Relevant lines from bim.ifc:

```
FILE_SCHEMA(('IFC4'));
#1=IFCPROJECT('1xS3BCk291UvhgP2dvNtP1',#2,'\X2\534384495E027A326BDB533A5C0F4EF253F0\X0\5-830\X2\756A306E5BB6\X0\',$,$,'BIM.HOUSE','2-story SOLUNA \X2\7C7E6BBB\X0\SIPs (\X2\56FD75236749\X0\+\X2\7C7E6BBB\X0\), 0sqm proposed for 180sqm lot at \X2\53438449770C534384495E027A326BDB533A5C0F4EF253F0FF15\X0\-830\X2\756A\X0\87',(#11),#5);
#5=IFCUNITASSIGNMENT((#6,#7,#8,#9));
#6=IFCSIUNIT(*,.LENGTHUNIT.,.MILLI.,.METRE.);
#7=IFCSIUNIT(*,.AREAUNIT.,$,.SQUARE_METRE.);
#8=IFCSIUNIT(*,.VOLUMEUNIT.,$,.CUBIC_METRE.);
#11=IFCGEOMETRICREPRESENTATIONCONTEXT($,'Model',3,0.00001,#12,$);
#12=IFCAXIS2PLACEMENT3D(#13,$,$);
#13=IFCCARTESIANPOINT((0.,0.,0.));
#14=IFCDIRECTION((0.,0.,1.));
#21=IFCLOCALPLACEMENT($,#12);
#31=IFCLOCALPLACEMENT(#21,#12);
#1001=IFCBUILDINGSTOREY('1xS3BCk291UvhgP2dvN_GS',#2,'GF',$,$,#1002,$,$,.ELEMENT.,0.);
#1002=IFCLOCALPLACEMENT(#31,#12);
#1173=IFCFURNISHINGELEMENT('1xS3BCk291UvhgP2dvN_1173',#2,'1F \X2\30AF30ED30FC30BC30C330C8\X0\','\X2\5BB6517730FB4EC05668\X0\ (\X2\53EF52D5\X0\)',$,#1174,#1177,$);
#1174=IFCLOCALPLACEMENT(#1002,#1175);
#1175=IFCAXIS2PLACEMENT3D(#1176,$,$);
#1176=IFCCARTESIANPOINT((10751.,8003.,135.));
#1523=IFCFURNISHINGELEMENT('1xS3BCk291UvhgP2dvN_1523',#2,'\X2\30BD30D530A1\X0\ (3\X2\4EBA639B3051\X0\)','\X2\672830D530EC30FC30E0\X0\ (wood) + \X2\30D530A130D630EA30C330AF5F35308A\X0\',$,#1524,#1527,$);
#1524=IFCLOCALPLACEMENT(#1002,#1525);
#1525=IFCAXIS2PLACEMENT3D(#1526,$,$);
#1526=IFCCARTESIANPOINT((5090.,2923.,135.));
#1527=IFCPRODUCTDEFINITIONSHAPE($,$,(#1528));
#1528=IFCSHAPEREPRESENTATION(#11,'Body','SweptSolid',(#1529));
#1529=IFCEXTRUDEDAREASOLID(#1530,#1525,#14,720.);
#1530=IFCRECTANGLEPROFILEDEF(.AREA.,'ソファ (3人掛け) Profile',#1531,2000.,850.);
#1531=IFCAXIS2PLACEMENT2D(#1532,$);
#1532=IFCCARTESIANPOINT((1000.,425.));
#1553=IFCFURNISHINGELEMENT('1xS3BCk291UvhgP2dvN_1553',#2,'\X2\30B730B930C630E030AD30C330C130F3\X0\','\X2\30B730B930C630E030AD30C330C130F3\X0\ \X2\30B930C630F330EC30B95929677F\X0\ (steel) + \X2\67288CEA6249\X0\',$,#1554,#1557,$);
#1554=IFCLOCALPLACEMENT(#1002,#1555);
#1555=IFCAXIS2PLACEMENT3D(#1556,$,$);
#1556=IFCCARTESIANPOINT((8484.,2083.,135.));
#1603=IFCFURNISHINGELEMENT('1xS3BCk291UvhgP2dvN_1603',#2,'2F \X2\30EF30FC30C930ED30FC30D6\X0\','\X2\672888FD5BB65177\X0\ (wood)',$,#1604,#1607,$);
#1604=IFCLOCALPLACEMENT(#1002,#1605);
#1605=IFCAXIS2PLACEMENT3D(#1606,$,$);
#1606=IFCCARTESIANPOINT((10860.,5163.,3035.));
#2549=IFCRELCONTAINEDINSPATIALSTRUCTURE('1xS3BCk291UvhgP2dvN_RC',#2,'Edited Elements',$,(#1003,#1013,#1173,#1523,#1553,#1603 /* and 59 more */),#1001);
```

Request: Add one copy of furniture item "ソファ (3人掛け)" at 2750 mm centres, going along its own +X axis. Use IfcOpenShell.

```python
import ifcopenshell
import ifcopenshell.api.geometry
import ifcopenshell.api.root
import ifcopenshell.util.element
import ifcopenshell.util.placement

model = ifcopenshell.open("bim.ifc")


def reuse_history(source, copy):
    """copy_class also copies each property set's owner history, people and application; keep the originals."""
    for rel in copy.IsDefinedBy:
        if rel.is_a("IfcRelDefinesByProperties") and (history := rel.RelatingPropertyDefinition.OwnerHistory):
            rel.RelatingPropertyDefinition.OwnerHistory = source.OwnerHistory
            ifcopenshell.util.element.remove_deep2(model, history)


source = model.by_guid("1xS3BCk291UvhgP2dvN_1523")
base = ifcopenshell.util.placement.get_local_placement(source.ObjectPlacement)
step = base[:3, 0] * 2750.0

for i in range(1, 2):
    copy = ifcopenshell.api.root.copy_class(model, product=source)
    copy.Representation = ifcopenshell.util.element.copy_deep(
        model, source.Representation, exclude=["IfcGeometricRepresentationContext", "IfcRepresentationMap"]
    )
    reuse_history(source, copy)
    matrix = base.copy()
    matrix[:3, 3] += i * step
    print("added at", matrix[:3, 3].round(3) + 0.0)
    ifcopenshell.api.geometry.edit_object_placement(model, product=copy, matrix=matrix, is_si=False)

model.write("bim-out.ifc")
```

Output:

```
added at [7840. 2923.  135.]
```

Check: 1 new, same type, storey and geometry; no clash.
